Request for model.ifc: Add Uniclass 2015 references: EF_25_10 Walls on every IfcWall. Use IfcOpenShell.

First a look at what the model holds.

```python
import ifcopenshell

model = ifcopenshell.open("model.ifc")
print(model.schema)
print("classifications:", [c.Name for c in model.by_type("IfcClassification")])
for ifc_class in ("IfcDoor", "IfcRoof", "IfcStair", "IfcWall", "IfcWindow"):
    print(ifc_class, len(model.by_type(ifc_class)))
```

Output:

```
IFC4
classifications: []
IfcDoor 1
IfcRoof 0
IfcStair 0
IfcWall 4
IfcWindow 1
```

```python
import ifcopenshell
import ifcopenshell.api.classification

model = ifcopenshell.open("model.ifc")

system = ifcopenshell.api.classification.add_classification(model, classification="Uniclass 2015")

codes = {
    "IfcWall": ("EF_25_10", "Walls"),
}
for ifc_class, (code, name) in codes.items():
    products = model.by_type(ifc_class)
    ifcopenshell.api.classification.add_reference(
        model, products=products, classification=system, identification=code, name=name
    )
    print(code, len(products))

model.write("model_rev.ifc")
```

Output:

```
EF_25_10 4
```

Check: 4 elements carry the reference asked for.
